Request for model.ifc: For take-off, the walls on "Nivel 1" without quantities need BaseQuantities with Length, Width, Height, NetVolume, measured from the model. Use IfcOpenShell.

First a look at what the model holds.

```python
import ifcopenshell
import ifcopenshell.util.element
import ifcopenshell.util.unit

model = ifcopenshell.open("model.ifc")
print(model.schema)
for unit_type in ("LENGTHUNIT", "AREAUNIT", "VOLUMEUNIT"):
    print(unit_type, ifcopenshell.util.unit.calculate_unit_scale(model, unit_type))
storey = next(s for s in model.by_type("IfcBuildingStorey") if s.Name == "Nivel 1")
walls = [e for e in ifcopenshell.util.element.get_decomposition(storey) if e.is_a("IfcWall")]
for e in sorted(walls, key=lambda e: e.id()):
    print(e.id(), e.is_a(), e.Name, list(ifcopenshell.util.element.get_psets(e, qtos_only=True)), sep=" | ")
```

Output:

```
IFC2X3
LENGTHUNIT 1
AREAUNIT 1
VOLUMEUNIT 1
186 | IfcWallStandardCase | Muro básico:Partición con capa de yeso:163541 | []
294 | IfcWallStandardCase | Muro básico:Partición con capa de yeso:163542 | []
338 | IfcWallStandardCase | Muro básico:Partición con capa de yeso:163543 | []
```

```python
import ifcopenshell
import ifcopenshell.api.pset
import ifcopenshell.geom
import ifcopenshell.util.element
import ifcopenshell.util.shape
import ifcopenshell.util.unit

model = ifcopenshell.open("model.ifc")
unit_scale = ifcopenshell.util.unit.calculate_unit_scale(model)
volume_scale = ifcopenshell.util.unit.calculate_unit_scale(model, "VOLUMEUNIT")
settings = ifcopenshell.geom.settings()

storey = next(s for s in model.by_type("IfcBuildingStorey") if s.Name == "Nivel 1")
walls = [e for e in ifcopenshell.util.element.get_decomposition(storey) if e.is_a("IfcWall")]

for e in sorted(walls, key=lambda e: e.id()):
    if ifcopenshell.util.element.get_psets(e, qtos_only=True, should_inherit=False):
        continue
    # Geometry comes back in metres, in the element's own axes.
    shape = ifcopenshell.geom.create_shape(settings, e)
    values = {
        "Length": ifcopenshell.util.shape.get_x(shape.geometry) / unit_scale,
        "Width": ifcopenshell.util.shape.get_y(shape.geometry) / unit_scale,
        "Height": ifcopenshell.util.shape.get_z(shape.geometry) / unit_scale,
        "NetVolume": ifcopenshell.util.shape.get_volume(shape.geometry) / volume_scale,
    }
    qto = ifcopenshell.api.pset.add_qto(model, product=e, name="BaseQuantities")
    ifcopenshell.api.pset.edit_qto(model, qto=qto, properties=values)
    print(e.id(), {k: round(v, 3) for k, v in values.items()})

model.write("model_updated.ifc")
```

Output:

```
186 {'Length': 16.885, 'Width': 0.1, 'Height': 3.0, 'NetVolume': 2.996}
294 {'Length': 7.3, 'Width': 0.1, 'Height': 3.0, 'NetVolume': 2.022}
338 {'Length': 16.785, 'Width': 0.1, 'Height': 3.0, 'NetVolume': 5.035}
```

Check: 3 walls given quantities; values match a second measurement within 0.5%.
